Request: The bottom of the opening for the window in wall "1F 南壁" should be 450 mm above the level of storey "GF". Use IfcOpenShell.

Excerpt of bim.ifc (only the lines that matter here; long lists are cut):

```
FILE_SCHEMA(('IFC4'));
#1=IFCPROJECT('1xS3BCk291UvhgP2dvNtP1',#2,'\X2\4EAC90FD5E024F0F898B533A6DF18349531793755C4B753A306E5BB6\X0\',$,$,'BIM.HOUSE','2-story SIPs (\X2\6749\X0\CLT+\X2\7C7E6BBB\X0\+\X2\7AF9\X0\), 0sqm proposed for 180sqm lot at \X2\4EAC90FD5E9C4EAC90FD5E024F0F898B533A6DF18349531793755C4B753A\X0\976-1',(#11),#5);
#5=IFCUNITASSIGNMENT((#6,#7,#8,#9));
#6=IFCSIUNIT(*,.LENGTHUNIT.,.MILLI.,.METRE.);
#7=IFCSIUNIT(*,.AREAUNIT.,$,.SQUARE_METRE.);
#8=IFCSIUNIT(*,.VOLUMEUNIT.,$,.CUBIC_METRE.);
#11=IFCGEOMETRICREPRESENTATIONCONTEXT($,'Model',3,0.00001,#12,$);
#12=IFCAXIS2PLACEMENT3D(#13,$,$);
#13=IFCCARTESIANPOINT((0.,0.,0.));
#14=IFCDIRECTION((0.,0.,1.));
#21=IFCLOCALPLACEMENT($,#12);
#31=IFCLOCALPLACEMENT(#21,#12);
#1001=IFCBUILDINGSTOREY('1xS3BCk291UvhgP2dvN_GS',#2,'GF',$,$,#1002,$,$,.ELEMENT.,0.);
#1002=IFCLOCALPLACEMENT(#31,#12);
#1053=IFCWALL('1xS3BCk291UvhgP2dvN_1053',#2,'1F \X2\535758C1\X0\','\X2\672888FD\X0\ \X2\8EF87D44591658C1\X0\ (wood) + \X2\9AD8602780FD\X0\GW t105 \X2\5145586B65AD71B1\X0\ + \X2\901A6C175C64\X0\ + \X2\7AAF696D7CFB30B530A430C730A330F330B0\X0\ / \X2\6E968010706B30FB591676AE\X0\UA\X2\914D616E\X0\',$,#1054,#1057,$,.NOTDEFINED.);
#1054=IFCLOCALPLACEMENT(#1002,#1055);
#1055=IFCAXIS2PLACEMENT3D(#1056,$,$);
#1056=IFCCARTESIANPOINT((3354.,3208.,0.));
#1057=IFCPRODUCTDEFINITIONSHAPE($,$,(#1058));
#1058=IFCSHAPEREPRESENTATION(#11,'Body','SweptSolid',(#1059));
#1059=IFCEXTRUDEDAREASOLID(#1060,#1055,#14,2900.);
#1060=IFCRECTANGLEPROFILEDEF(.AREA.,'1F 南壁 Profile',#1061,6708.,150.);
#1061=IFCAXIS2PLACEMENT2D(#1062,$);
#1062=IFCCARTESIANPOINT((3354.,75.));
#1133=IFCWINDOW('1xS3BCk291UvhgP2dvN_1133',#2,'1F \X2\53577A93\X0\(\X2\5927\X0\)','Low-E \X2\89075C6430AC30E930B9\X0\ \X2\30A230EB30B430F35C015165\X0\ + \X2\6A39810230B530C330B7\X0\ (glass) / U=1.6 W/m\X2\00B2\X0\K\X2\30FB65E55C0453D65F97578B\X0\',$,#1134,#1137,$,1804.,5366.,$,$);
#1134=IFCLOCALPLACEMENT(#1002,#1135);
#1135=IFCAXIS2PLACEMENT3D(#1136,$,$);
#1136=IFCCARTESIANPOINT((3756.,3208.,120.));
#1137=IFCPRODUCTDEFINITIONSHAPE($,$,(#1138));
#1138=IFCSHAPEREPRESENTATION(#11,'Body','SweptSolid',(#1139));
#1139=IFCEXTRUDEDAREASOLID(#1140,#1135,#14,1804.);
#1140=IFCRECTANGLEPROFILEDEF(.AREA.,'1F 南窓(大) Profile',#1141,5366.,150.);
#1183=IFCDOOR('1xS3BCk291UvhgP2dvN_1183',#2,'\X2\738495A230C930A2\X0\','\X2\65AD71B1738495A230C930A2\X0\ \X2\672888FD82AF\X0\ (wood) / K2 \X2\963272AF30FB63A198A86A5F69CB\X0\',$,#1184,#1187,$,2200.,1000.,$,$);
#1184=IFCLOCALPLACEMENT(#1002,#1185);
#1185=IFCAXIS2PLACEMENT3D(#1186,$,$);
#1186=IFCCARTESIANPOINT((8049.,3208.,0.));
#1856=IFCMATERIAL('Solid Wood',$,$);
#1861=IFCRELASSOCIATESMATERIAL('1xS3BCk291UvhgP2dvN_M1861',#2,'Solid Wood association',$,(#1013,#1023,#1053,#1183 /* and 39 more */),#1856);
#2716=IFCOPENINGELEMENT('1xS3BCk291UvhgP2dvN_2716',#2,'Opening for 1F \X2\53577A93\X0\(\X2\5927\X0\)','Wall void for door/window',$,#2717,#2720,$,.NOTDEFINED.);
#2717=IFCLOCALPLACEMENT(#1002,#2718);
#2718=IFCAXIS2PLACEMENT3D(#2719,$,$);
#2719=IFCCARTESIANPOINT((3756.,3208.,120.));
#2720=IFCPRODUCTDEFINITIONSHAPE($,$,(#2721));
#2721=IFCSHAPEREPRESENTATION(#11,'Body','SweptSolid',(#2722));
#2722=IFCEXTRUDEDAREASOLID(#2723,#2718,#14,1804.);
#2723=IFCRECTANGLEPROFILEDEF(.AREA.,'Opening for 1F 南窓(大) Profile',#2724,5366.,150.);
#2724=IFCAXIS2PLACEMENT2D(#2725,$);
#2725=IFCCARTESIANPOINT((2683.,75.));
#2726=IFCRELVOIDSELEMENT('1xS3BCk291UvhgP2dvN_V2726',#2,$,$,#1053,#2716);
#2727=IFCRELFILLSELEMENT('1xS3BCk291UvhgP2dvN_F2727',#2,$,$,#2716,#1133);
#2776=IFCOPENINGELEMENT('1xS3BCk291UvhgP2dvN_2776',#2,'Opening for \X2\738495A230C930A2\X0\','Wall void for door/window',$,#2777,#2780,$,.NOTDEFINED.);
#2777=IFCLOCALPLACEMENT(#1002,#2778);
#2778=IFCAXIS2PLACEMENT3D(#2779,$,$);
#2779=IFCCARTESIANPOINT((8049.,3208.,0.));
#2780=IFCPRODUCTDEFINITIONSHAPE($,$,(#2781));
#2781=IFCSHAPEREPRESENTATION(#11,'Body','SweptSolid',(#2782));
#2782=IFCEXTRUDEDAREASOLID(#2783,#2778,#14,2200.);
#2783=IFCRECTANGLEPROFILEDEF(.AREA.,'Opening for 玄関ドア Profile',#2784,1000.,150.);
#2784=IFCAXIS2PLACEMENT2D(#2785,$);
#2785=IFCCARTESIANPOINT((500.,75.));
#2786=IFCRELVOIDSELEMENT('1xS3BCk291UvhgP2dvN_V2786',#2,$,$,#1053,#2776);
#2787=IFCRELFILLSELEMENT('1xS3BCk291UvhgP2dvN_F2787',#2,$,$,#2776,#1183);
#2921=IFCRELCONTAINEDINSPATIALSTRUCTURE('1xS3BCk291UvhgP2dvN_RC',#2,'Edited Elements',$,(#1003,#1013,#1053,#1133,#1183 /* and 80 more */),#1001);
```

```python
import numpy as np
import ifcopenshell
import ifcopenshell.api.geometry
import ifcopenshell.geom
import ifcopenshell.util.element
import ifcopenshell.util.placement
import ifcopenshell.util.shape
import ifcopenshell.util.unit

model = ifcopenshell.open("bim.ifc")
unit_scale = ifcopenshell.util.unit.calculate_unit_scale(model)

window = model.by_guid("1xS3BCk291UvhgP2dvN_1133")
opening = window.FillsVoids[0].RelatingOpeningElement
storey = ifcopenshell.util.element.get_container(window, ifc_class="IfcBuildingStorey")
level = ifcopenshell.util.placement.get_local_placement(storey.ObjectPlacement)[2, 3]

# The opening's origin need not be at the sill, so measure its lowest point.
shape = ifcopenshell.geom.create_shape(ifcopenshell.geom.settings(), opening)
bottom = ifcopenshell.util.shape.get_shape_bottom_elevation(shape, shape.geometry) / unit_scale
dz = level + 0.45 / unit_scale - bottom

shift = np.array([0.0, 0.0, dz])
# The window is not placed relative to its opening, so move both.
for product in (opening, window):
    matrix = ifcopenshell.util.placement.get_local_placement(product.ObjectPlacement)
    matrix[:3, 3] += shift
    ifcopenshell.api.geometry.edit_object_placement(model, product=product, matrix=matrix, is_si=False)

print(f"moved by {dz * unit_scale:+.3f} m")

model.write("bim_rev.ifc")
```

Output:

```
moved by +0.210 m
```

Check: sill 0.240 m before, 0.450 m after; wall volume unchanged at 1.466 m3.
